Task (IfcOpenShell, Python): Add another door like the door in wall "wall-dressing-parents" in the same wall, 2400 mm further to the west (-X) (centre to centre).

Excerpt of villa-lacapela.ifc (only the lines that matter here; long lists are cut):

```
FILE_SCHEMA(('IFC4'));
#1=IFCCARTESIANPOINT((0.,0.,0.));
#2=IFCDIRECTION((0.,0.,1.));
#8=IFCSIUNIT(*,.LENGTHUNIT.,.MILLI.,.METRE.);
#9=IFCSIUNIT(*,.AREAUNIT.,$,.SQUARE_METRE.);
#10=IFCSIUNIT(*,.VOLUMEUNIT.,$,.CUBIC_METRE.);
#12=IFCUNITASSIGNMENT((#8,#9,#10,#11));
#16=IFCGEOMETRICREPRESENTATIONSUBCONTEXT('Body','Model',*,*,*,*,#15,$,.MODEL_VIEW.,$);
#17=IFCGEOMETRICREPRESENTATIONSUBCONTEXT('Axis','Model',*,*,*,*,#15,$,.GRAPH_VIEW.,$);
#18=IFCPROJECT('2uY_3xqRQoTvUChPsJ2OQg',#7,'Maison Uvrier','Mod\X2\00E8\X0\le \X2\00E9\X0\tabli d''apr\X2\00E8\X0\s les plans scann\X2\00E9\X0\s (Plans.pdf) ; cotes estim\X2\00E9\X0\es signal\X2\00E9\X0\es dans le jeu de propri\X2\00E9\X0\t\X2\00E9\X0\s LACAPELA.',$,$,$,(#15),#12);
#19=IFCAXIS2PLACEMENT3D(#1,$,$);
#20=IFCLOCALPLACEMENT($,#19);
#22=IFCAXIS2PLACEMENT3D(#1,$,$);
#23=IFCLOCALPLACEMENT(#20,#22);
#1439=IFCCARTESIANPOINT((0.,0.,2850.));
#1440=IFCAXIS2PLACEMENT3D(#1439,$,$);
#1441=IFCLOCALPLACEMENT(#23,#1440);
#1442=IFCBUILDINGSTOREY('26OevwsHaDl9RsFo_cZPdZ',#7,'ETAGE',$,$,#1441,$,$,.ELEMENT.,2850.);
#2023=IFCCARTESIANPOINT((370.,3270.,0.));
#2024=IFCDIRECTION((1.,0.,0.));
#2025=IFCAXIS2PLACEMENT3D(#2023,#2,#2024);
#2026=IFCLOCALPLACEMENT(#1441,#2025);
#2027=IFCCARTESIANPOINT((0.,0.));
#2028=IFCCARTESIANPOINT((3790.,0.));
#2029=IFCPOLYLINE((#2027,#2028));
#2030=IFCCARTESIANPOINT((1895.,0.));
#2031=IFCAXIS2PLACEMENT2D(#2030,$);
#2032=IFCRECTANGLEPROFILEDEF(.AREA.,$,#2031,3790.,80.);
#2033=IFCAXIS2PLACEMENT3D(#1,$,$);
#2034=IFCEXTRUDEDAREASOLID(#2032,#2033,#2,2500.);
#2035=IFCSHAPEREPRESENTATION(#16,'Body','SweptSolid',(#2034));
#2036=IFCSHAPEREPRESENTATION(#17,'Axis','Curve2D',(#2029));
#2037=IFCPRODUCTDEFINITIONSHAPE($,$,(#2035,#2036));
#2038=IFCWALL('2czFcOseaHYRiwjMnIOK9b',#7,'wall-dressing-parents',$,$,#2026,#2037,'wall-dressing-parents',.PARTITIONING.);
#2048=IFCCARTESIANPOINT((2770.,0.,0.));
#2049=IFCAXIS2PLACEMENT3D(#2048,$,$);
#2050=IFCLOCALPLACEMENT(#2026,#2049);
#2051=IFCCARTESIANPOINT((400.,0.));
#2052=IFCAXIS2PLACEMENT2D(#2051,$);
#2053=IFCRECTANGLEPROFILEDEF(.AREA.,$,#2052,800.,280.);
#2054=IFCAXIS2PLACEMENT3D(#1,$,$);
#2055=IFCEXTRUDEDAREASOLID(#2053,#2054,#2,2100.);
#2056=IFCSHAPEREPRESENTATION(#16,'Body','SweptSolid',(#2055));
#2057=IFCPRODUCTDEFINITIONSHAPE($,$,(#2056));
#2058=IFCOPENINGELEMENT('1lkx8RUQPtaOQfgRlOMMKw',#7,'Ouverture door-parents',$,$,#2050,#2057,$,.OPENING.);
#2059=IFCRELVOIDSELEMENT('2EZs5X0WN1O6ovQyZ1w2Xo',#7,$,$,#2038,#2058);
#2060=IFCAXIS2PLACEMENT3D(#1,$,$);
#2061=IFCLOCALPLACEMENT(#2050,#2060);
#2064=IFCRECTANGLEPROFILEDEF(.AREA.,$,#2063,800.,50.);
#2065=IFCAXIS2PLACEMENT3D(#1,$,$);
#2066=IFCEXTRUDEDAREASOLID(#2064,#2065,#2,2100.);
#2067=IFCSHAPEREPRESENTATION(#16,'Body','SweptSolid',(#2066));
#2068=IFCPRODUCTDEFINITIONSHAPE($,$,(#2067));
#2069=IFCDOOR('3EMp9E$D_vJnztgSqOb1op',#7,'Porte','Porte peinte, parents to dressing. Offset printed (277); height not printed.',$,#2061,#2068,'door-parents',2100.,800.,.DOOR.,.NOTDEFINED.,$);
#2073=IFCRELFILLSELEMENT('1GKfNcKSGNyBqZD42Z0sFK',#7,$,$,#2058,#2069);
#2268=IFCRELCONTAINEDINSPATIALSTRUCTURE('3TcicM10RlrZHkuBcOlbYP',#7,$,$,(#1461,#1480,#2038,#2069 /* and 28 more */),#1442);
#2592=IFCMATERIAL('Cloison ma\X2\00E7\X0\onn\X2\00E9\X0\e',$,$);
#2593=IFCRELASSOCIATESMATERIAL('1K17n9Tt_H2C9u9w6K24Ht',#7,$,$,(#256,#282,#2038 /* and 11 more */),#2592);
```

```python
import ifcopenshell
import ifcopenshell.api.feature
import ifcopenshell.api.geometry
import ifcopenshell.api.root
import ifcopenshell.geom
import ifcopenshell.util.element
import ifcopenshell.util.placement
import ifcopenshell.util.shape

model = ifcopenshell.open("villa-lacapela.ifc")
settings = ifcopenshell.geom.settings()


def volume(element):
    """Net volume in cubic metres, openings subtracted."""
    shape = ifcopenshell.geom.create_shape(settings, element)
    return ifcopenshell.util.shape.get_volume(shape.geometry)


def reuse_history(source, copy):
    """copy_class also copies each property set's owner history, people and application; keep the originals."""
    for rel in copy.IsDefinedBy:
        if rel.is_a("IfcRelDefinesByProperties") and (history := rel.RelatingPropertyDefinition.OwnerHistory):
            rel.RelatingPropertyDefinition.OwnerHistory = source.OwnerHistory
            ifcopenshell.util.element.remove_deep2(model, history)


door = model.by_guid("3EMp9E$D_vJnztgSqOb1op")
opening = door.FillsVoids[0].RelatingOpeningElement
wall = opening.VoidsElements[0].RelatingBuildingElement
before = volume(wall)
shift = ifcopenshell.util.placement.get_local_placement(wall.ObjectPlacement)[:3, 0] * -2400.0

# copy_class copies the void relationship, type, container and properties, but no geometry.
new_opening = ifcopenshell.api.root.copy_class(model, product=opening)
new_opening.Representation = ifcopenshell.util.element.copy_deep(
    model, opening.Representation, exclude=["IfcGeometricRepresentationContext", "IfcRepresentationMap"]
)
new_door = ifcopenshell.api.root.copy_class(model, product=door)
new_door.Representation = ifcopenshell.util.element.copy_deep(
    model, door.Representation, exclude=["IfcGeometricRepresentationContext", "IfcRepresentationMap"]
)
new_door.Tag = None
reuse_history(door, new_door)
ifcopenshell.api.feature.add_filling(model, opening=new_opening, element=new_door)

for old, new in ((opening, new_opening), (door, new_door)):
    matrix = ifcopenshell.util.placement.get_local_placement(old.ObjectPlacement)
    matrix[:3, 3] += shift
    ifcopenshell.api.geometry.edit_object_placement(model, product=new, matrix=matrix, is_si=False)

after = volume(wall)

print(f"wall volume {before:.3f} -> {after:.3f} m3")

model.write("villa-lacapela_v2.ifc")
```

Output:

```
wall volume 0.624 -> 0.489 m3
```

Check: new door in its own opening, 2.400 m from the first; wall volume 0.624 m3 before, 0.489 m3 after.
